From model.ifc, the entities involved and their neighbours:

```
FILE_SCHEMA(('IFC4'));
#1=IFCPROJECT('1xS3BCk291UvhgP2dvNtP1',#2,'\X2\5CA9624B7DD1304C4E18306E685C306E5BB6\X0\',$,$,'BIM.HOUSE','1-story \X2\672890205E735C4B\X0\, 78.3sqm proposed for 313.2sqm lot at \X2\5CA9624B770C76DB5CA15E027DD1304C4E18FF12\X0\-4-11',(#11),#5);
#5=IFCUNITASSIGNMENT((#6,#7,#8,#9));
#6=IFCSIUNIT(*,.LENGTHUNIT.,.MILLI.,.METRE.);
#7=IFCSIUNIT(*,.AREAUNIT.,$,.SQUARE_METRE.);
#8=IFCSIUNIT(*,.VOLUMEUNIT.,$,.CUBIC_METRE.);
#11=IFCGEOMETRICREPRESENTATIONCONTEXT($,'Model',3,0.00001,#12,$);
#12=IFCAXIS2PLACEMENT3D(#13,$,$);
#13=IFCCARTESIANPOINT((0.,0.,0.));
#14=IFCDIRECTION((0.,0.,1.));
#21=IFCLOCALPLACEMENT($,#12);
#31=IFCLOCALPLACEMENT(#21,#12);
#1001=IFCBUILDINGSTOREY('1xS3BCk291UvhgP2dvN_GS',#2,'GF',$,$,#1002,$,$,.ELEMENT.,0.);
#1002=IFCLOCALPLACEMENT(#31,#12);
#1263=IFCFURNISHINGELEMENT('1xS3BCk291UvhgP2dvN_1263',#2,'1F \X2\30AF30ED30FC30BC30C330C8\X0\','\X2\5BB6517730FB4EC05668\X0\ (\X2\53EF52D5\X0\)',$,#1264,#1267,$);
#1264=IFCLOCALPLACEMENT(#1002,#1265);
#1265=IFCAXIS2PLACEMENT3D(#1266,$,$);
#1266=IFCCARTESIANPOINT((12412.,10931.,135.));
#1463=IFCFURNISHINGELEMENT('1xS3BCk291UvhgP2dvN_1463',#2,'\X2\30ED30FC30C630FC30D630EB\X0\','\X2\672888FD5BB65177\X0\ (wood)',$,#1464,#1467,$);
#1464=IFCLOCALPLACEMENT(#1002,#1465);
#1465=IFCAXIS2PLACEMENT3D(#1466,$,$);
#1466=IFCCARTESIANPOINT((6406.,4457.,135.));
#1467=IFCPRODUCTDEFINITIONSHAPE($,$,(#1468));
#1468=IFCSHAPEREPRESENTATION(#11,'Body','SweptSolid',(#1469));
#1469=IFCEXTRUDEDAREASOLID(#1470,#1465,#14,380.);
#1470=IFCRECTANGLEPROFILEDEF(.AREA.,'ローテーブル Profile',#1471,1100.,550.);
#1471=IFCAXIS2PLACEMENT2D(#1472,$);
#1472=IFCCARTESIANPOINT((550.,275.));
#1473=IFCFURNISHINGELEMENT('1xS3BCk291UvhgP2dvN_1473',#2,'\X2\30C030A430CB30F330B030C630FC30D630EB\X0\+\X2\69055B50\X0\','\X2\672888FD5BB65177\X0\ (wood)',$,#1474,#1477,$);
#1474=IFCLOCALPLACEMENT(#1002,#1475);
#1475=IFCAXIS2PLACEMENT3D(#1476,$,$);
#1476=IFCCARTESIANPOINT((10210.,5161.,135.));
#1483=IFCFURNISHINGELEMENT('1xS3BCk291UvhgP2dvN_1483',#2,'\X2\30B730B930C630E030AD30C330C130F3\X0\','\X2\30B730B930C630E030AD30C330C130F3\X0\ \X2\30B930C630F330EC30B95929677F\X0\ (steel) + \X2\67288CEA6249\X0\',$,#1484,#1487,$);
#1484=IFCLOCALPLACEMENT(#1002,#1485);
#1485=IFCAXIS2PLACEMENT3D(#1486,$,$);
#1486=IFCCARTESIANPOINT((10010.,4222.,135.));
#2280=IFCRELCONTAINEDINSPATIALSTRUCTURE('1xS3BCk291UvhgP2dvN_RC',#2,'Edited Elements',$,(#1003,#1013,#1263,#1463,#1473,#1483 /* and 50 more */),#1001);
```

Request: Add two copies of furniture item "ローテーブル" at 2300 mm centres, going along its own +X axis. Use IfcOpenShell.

```python
import ifcopenshell
import ifcopenshell.api.geometry
import ifcopenshell.api.root
import ifcopenshell.util.element
import ifcopenshell.util.placement
import ifcopenshell.util.unit

model = ifcopenshell.open("model.ifc")
unit_scale = ifcopenshell.util.unit.calculate_unit_scale(model)


def reuse_history(source, copy):
    """copy_class also copies each property set's owner history, people and application; keep the originals."""
    for rel in copy.IsDefinedBy:
        if rel.is_a("IfcRelDefinesByProperties") and (history := rel.RelatingPropertyDefinition.OwnerHistory):
            rel.RelatingPropertyDefinition.OwnerHistory = source.OwnerHistory
            ifcopenshell.util.element.remove_deep2(model, history)


source = model.by_guid("1xS3BCk291UvhgP2dvN_1463")
base = ifcopenshell.util.placement.get_local_placement(source.ObjectPlacement)
step = base[:3, 0] * 2.3 / unit_scale

for i in range(1, 3):
    copy = ifcopenshell.api.root.copy_class(model, product=source)
    copy.Representation = ifcopenshell.util.element.copy_deep(
        model, source.Representation, exclude=["IfcGeometricRepresentationContext", "IfcRepresentationMap"]
    )
    reuse_history(source, copy)
    matrix = base.copy()
    matrix[:3, 3] += i * step
    print("added at", matrix[:3, 3].round(3) + 0.0)
    ifcopenshell.api.geometry.edit_object_placement(model, product=copy, matrix=matrix, is_si=False)

model.write("model-out.ifc")
```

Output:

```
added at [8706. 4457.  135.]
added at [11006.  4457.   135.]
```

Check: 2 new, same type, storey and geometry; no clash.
